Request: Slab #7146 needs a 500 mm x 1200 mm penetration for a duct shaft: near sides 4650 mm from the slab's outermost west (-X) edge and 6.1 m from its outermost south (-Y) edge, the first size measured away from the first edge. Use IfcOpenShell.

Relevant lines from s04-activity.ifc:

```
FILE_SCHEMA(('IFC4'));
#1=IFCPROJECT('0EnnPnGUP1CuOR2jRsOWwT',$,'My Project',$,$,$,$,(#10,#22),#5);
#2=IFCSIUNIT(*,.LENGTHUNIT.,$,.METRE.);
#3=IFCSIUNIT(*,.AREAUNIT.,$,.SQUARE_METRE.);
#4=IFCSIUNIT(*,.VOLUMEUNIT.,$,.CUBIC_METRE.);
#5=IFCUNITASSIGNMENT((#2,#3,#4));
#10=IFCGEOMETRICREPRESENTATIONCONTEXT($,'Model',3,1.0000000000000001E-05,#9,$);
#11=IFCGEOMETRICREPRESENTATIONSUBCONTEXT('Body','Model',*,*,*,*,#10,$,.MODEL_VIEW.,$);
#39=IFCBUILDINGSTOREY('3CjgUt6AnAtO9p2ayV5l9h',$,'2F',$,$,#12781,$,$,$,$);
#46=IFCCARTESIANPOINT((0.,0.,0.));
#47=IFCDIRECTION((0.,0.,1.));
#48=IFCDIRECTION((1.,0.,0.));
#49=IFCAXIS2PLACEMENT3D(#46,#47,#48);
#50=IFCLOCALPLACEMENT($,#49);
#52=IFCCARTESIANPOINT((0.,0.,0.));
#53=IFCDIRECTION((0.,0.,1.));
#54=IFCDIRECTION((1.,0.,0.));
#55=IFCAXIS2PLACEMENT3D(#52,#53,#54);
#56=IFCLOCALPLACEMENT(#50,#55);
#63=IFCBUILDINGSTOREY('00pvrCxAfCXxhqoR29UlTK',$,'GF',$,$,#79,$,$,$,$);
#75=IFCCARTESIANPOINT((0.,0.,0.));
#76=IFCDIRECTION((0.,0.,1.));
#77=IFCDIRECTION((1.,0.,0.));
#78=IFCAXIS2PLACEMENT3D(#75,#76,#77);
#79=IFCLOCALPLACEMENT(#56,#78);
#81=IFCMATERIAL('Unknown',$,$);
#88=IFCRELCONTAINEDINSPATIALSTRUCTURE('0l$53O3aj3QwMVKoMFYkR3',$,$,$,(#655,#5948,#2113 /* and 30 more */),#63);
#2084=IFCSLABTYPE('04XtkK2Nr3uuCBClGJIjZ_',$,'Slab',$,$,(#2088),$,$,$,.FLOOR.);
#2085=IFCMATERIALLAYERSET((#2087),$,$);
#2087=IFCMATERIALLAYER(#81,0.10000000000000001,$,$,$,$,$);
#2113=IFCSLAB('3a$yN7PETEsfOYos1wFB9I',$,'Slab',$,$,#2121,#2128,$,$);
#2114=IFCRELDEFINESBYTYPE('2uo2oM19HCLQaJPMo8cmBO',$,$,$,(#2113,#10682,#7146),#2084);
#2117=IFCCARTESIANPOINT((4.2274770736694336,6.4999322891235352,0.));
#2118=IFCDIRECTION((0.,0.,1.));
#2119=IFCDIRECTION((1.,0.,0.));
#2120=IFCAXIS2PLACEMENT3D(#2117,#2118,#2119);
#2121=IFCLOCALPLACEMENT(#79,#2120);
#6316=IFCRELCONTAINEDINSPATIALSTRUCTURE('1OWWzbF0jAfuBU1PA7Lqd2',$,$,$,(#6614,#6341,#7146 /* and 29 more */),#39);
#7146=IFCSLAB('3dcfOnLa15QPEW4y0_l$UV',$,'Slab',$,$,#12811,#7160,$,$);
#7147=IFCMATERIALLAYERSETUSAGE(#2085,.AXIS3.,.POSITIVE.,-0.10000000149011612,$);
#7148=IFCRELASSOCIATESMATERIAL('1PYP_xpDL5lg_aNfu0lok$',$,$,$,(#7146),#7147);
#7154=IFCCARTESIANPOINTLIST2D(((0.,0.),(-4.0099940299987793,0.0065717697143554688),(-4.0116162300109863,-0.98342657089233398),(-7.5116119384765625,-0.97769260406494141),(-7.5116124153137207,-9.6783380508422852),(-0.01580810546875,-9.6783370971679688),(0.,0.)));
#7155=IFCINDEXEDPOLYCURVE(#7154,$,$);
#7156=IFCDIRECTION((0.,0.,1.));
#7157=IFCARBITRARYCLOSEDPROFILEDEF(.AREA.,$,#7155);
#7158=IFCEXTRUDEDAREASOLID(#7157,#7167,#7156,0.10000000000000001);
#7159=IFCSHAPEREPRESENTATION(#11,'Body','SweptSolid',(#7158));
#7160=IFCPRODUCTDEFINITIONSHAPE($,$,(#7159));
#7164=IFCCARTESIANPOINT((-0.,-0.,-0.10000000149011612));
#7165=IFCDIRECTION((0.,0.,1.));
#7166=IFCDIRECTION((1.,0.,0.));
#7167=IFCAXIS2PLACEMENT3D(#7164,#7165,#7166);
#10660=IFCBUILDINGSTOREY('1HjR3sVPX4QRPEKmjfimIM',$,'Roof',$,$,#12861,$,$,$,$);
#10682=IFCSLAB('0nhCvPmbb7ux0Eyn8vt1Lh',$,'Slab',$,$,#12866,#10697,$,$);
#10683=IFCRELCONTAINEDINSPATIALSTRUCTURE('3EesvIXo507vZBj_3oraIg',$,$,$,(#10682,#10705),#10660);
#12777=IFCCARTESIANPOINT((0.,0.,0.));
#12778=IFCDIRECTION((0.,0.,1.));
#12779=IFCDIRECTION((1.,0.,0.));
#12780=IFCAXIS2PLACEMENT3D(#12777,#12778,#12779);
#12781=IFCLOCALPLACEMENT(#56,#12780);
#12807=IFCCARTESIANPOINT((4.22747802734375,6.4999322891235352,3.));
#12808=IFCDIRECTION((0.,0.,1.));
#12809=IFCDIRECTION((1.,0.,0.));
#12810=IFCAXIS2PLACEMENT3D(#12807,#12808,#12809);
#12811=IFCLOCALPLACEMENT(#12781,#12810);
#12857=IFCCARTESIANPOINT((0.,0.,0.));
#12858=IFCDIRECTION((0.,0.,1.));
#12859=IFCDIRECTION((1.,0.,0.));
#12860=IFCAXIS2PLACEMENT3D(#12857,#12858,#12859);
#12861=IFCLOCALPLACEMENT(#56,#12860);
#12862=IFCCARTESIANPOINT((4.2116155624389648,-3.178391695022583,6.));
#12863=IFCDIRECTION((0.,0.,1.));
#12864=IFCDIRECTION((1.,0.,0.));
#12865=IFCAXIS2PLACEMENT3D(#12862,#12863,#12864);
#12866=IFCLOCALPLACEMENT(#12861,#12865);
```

```python
import numpy as np
import ifcopenshell
import ifcopenshell.api.feature
import ifcopenshell.api.geometry
import ifcopenshell.api.root
import ifcopenshell.geom
import ifcopenshell.util.placement
import ifcopenshell.util.representation
import ifcopenshell.util.shape
import ifcopenshell.util.unit

model = ifcopenshell.open("s04-activity.ifc")
unit_scale = ifcopenshell.util.unit.calculate_unit_scale(model)
settings = ifcopenshell.geom.settings()


def volume(element):
    """Net volume in cubic metres, openings subtracted."""
    shape = ifcopenshell.geom.create_shape(settings, element)
    return ifcopenshell.util.shape.get_volume(shape.geometry)


slab = model.by_guid("3dcfOnLa15QPEW4y0_l$UV")
before = volume(slab)

# Extent in the slab's own axes, in metres. The edges named are its -X and -Y sides.
slab_shape = ifcopenshell.geom.create_shape(settings, slab)
vertices = ifcopenshell.util.shape.get_vertices(slab_shape.geometry)
x_min, y_min, bottom = vertices.min(axis=0)
top = vertices[:, 2].max()

opening = ifcopenshell.api.root.create_entity(model, ifc_class="IfcOpeningElement", name="Duct shaft opening", predefined_type="OPENING")
context = ifcopenshell.util.representation.get_context(model, "Model", "Body", "MODEL_VIEW")
width, depth = 0.5, 1.2
outline = [(0.0, 0.0), (width, 0.0), (width, depth), (0.0, depth), (0.0, 0.0)]
# Overshoot both faces by 50 mm so the cut is clean.
shape = ifcopenshell.api.geometry.add_slab_representation(
    model, context=context, depth=top - bottom + 0.1, polyline=outline
)
ifcopenshell.api.geometry.assign_representation(model, product=opening, representation=shape)

matrix = ifcopenshell.util.placement.get_local_placement(slab.ObjectPlacement)
matrix[:, 3] = matrix @ np.append(np.array([x_min + 4.65, y_min + 6.1, bottom - 0.05]) / unit_scale, 1.0)
ifcopenshell.api.geometry.edit_object_placement(model, product=opening, matrix=matrix, is_si=False)
ifcopenshell.api.feature.add_feature(model, feature=opening, element=slab)

after = volume(slab)

print(f"slab volume {before:.3f} -> {after:.3f} m3")

model.write("s04-activity-out.ifc")
```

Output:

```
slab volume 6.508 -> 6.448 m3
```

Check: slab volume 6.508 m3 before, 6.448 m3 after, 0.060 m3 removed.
